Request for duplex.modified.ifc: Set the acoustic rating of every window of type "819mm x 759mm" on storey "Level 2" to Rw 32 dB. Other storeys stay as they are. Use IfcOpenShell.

First a look at what the model holds.

```python
import ifcopenshell
import ifcopenshell.util.element

model = ifcopenshell.open("duplex.modified.ifc")
print(model.schema)
storey = next(s for s in model.by_type("IfcBuildingStorey") if s.Name == "Level 2")
windows = [e for e in ifcopenshell.util.element.get_decomposition(storey) if e.is_a("IfcWindow")]
seen = {}
for e in windows:
    element_type = ifcopenshell.util.element.get_type(e)
    key = (element_type.Name if element_type != e and element_type else None, ifcopenshell.util.element.get_pset(e, "Pset_WindowCommon", "AcousticRating"))
    seen[key] = seen.get(key, 0) + 1
for (name, value), count in sorted(seen.items(), key=str):
    print(count, "x", name, "|", value)
```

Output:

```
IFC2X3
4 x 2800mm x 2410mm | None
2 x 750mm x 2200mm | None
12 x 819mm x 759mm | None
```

```python
import ifcopenshell
import ifcopenshell.api.pset
import ifcopenshell.util.element

model = ifcopenshell.open("duplex.modified.ifc")

storey = next(s for s in model.by_type("IfcBuildingStorey") if s.Name == "Level 2")
windows = [e for e in ifcopenshell.util.element.get_decomposition(storey) if e.is_a("IfcWindow")]

count = 0
for e in windows:
    element_type = ifcopenshell.util.element.get_type(e)
    if element_type in (None, e) or element_type.Name != "819mm x 759mm":
        continue
    # add_pset returns the element's existing set when there is one.
    pset = ifcopenshell.api.pset.add_pset(model, product=e, name="Pset_WindowCommon")
    ifcopenshell.api.pset.edit_pset(model, pset=pset, properties={"AcousticRating": "Rw 32 dB"})
    count += 1

print(count, "windows updated")

model.write("duplex.modified_rev.ifc")
```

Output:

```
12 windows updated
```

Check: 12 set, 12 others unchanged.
